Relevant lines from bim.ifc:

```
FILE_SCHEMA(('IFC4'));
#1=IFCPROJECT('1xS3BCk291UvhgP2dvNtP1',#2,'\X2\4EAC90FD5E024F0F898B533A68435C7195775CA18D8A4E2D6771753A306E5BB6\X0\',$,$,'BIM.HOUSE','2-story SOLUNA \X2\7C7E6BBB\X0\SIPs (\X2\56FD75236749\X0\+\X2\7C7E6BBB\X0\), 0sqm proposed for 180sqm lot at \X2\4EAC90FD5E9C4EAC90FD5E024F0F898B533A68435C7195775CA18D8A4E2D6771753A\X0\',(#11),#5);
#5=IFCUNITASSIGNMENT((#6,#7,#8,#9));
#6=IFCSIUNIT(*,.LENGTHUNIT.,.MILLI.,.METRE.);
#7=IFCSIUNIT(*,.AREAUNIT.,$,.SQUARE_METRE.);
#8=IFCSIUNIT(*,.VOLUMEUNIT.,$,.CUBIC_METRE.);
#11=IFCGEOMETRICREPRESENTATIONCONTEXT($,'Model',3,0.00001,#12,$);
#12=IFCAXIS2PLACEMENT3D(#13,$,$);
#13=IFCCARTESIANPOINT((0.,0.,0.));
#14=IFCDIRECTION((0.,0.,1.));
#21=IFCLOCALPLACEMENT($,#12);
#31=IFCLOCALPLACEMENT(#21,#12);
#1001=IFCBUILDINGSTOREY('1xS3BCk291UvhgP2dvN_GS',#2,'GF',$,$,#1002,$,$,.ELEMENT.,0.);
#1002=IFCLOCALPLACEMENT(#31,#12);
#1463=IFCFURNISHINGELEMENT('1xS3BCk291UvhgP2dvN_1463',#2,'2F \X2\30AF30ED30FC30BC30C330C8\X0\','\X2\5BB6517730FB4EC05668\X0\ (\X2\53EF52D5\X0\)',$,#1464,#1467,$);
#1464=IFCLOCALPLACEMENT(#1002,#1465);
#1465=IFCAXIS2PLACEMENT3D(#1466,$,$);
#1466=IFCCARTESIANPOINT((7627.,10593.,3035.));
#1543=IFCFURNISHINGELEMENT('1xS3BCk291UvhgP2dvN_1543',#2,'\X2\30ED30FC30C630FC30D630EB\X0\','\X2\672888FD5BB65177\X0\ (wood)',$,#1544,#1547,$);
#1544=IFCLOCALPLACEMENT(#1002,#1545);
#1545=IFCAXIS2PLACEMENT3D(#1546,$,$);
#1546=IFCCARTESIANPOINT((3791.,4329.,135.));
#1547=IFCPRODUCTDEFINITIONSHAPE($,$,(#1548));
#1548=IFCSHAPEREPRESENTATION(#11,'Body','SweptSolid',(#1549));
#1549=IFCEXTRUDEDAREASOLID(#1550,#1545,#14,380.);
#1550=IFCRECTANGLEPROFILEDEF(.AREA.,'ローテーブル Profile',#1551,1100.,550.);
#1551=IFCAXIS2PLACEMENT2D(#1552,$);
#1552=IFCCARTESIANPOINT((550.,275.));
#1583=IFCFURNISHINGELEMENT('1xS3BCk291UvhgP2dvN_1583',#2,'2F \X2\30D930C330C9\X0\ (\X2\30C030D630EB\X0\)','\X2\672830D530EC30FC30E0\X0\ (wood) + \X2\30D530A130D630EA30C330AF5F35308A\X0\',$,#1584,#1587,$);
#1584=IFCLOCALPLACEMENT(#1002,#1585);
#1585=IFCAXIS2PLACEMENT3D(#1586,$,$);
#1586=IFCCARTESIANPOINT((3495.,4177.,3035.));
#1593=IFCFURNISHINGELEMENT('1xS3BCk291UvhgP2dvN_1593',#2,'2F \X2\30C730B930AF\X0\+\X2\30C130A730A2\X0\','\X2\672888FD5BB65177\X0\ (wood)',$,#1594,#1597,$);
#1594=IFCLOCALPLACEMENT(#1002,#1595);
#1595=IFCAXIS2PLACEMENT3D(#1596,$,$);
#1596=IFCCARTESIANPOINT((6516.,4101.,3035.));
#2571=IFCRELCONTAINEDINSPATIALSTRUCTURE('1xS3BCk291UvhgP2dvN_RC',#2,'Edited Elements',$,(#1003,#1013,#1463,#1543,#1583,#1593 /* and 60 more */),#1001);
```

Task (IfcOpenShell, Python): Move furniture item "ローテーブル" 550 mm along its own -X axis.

```python
import ifcopenshell
import ifcopenshell.api.geometry
import ifcopenshell.util.placement

model = ifcopenshell.open("bim.ifc")

item = model.by_id(1543)
matrix = ifcopenshell.util.placement.get_local_placement(item.ObjectPlacement)
matrix[:3, 3] -= matrix[:3, 0] * 550.0
ifcopenshell.api.geometry.edit_object_placement(model, product=item, matrix=matrix, is_si=False)

print(ifcopenshell.util.placement.get_local_placement(item.ObjectPlacement).round(3) + 0.0)

model.write("bim_rev.ifc")
```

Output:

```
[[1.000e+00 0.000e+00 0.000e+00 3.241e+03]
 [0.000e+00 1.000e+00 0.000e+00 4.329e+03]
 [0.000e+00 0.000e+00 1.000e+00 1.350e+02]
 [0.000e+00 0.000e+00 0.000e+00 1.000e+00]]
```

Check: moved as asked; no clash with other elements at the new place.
